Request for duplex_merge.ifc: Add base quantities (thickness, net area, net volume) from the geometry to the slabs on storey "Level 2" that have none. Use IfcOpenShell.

First a look at what the model holds.

```python
import ifcopenshell
import ifcopenshell.util.element
import ifcopenshell.util.unit

model = ifcopenshell.open("duplex_merge.ifc")
print(model.schema)
for unit_type in ("LENGTHUNIT", "AREAUNIT", "VOLUMEUNIT"):
    print(unit_type, ifcopenshell.util.unit.calculate_unit_scale(model, unit_type))
storey = next(s for s in model.by_type("IfcBuildingStorey") if s.Name == "Level 2")
slabs = [e for e in ifcopenshell.util.element.get_decomposition(storey) if e.is_a("IfcSlab")]
for e in sorted(slabs, key=lambda e: e.id()):
    print(e.id(), e.is_a(), e.Name, list(ifcopenshell.util.element.get_psets(e, qtos_only=True)), sep=" | ")
```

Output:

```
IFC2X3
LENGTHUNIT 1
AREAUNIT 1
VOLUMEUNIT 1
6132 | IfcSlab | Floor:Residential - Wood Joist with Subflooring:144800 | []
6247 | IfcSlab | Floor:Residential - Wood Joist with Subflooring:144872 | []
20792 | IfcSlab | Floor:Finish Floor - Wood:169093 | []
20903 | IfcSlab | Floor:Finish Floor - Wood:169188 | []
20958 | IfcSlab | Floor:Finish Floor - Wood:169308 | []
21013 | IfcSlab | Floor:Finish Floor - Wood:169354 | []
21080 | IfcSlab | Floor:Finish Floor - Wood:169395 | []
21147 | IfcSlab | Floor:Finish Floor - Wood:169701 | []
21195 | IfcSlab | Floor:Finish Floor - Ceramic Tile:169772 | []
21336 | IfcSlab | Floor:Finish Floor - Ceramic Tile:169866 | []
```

```python
import ifcopenshell
import ifcopenshell.api.pset
import ifcopenshell.geom
import ifcopenshell.util.element
import ifcopenshell.util.shape
import ifcopenshell.util.unit

model = ifcopenshell.open("duplex_merge.ifc")
unit_scale = ifcopenshell.util.unit.calculate_unit_scale(model)
area_scale = ifcopenshell.util.unit.calculate_unit_scale(model, "AREAUNIT")
volume_scale = ifcopenshell.util.unit.calculate_unit_scale(model, "VOLUMEUNIT")
settings = ifcopenshell.geom.settings()

storey = next(s for s in model.by_type("IfcBuildingStorey") if s.Name == "Level 2")
slabs = [e for e in ifcopenshell.util.element.get_decomposition(storey) if e.is_a("IfcSlab")]

for e in sorted(slabs, key=lambda e: e.id()):
    if ifcopenshell.util.element.get_psets(e, qtos_only=True, should_inherit=False):
        continue
    # Geometry comes back in metres, in the element's own axes.
    shape = ifcopenshell.geom.create_shape(settings, e)
    values = {
        "Width": ifcopenshell.util.shape.get_z(shape.geometry) / unit_scale,
        "NetArea": ifcopenshell.util.shape.get_footprint_area(shape.geometry) / area_scale,
        "NetVolume": ifcopenshell.util.shape.get_volume(shape.geometry) / volume_scale,
    }
    qto = ifcopenshell.api.pset.add_qto(model, product=e, name="BaseQuantities")
    ifcopenshell.api.pset.edit_qto(model, qto=qto, properties=values)
    print(e.id(), {k: round(v, 3) for k, v in values.items()})

model.write("duplex_merge_rev.ifc")
```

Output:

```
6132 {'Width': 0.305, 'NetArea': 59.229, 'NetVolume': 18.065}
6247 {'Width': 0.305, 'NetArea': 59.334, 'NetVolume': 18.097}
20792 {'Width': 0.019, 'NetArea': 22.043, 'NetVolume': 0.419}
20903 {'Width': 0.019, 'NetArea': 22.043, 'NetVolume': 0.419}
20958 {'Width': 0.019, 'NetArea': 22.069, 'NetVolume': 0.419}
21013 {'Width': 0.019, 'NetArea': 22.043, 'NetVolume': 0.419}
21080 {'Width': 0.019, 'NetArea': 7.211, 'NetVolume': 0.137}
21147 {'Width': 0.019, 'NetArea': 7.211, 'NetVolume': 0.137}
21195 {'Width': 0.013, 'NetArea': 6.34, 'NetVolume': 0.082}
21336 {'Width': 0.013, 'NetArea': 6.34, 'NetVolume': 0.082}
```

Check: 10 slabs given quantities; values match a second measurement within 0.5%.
